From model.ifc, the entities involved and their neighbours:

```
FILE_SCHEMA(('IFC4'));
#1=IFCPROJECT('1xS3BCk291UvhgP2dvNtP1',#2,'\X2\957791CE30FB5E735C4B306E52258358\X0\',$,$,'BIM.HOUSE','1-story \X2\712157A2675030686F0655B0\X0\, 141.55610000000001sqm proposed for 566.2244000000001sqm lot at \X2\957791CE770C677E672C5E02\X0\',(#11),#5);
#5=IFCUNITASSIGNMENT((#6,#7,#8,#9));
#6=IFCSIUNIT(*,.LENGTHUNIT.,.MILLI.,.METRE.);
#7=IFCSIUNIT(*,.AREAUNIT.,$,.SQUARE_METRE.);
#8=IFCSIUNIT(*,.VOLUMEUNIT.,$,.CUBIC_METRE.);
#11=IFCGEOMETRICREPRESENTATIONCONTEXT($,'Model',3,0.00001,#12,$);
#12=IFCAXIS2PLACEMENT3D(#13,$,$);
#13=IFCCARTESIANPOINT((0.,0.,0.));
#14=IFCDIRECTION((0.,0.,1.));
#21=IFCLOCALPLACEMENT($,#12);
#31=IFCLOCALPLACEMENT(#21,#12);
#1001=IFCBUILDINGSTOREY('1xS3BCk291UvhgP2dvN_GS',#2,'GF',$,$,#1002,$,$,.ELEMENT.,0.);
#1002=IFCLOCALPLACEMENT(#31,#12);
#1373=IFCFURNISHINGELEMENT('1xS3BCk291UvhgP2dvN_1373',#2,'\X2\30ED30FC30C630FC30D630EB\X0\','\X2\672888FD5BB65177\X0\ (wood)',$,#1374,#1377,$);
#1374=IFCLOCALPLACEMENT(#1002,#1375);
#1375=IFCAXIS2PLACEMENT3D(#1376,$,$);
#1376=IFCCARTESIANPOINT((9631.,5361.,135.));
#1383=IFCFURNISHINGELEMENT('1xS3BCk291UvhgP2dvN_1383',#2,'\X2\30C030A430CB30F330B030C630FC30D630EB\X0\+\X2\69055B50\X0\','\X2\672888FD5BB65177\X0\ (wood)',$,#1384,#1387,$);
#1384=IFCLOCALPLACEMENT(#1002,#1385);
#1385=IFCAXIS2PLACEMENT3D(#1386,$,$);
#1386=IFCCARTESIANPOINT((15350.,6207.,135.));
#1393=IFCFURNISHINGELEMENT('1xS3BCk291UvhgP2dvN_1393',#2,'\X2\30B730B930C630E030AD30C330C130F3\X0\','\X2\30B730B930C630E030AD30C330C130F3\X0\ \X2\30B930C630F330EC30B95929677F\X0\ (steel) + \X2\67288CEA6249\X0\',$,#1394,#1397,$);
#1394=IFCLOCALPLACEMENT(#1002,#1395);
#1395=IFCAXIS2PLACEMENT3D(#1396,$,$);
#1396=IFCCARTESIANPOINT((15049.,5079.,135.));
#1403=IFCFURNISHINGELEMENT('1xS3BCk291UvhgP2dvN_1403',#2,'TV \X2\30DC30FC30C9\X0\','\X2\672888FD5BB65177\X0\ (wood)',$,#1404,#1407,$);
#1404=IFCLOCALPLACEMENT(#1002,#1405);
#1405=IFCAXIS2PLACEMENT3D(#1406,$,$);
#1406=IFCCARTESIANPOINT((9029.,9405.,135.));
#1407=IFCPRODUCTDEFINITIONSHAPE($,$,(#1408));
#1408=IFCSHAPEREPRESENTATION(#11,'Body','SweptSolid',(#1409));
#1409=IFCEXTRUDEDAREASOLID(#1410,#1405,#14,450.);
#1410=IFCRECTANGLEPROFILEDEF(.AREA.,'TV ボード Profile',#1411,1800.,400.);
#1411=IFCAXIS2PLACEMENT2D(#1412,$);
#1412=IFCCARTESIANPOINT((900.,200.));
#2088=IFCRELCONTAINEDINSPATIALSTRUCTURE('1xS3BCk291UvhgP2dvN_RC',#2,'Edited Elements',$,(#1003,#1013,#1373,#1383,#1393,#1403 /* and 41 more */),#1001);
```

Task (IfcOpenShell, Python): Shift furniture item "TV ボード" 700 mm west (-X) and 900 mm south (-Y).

```python
import ifcopenshell
import ifcopenshell.api.geometry
import ifcopenshell.util.placement
import ifcopenshell.util.unit

model = ifcopenshell.open("model.ifc")
unit_scale = ifcopenshell.util.unit.calculate_unit_scale(model)

item = model.by_guid("1xS3BCk291UvhgP2dvN_1403")
matrix = ifcopenshell.util.placement.get_local_placement(item.ObjectPlacement)
matrix[0, 3] -= 0.7 / unit_scale
matrix[1, 3] -= 0.9 / unit_scale
ifcopenshell.api.geometry.edit_object_placement(model, product=item, matrix=matrix, is_si=False)

print(ifcopenshell.util.placement.get_local_placement(item.ObjectPlacement).round(3) + 0.0)

model.write("model-out.ifc")
```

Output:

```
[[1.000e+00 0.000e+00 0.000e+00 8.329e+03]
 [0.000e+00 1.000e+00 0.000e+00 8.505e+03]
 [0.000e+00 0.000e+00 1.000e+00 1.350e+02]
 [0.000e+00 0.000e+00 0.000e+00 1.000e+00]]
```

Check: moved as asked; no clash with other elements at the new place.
